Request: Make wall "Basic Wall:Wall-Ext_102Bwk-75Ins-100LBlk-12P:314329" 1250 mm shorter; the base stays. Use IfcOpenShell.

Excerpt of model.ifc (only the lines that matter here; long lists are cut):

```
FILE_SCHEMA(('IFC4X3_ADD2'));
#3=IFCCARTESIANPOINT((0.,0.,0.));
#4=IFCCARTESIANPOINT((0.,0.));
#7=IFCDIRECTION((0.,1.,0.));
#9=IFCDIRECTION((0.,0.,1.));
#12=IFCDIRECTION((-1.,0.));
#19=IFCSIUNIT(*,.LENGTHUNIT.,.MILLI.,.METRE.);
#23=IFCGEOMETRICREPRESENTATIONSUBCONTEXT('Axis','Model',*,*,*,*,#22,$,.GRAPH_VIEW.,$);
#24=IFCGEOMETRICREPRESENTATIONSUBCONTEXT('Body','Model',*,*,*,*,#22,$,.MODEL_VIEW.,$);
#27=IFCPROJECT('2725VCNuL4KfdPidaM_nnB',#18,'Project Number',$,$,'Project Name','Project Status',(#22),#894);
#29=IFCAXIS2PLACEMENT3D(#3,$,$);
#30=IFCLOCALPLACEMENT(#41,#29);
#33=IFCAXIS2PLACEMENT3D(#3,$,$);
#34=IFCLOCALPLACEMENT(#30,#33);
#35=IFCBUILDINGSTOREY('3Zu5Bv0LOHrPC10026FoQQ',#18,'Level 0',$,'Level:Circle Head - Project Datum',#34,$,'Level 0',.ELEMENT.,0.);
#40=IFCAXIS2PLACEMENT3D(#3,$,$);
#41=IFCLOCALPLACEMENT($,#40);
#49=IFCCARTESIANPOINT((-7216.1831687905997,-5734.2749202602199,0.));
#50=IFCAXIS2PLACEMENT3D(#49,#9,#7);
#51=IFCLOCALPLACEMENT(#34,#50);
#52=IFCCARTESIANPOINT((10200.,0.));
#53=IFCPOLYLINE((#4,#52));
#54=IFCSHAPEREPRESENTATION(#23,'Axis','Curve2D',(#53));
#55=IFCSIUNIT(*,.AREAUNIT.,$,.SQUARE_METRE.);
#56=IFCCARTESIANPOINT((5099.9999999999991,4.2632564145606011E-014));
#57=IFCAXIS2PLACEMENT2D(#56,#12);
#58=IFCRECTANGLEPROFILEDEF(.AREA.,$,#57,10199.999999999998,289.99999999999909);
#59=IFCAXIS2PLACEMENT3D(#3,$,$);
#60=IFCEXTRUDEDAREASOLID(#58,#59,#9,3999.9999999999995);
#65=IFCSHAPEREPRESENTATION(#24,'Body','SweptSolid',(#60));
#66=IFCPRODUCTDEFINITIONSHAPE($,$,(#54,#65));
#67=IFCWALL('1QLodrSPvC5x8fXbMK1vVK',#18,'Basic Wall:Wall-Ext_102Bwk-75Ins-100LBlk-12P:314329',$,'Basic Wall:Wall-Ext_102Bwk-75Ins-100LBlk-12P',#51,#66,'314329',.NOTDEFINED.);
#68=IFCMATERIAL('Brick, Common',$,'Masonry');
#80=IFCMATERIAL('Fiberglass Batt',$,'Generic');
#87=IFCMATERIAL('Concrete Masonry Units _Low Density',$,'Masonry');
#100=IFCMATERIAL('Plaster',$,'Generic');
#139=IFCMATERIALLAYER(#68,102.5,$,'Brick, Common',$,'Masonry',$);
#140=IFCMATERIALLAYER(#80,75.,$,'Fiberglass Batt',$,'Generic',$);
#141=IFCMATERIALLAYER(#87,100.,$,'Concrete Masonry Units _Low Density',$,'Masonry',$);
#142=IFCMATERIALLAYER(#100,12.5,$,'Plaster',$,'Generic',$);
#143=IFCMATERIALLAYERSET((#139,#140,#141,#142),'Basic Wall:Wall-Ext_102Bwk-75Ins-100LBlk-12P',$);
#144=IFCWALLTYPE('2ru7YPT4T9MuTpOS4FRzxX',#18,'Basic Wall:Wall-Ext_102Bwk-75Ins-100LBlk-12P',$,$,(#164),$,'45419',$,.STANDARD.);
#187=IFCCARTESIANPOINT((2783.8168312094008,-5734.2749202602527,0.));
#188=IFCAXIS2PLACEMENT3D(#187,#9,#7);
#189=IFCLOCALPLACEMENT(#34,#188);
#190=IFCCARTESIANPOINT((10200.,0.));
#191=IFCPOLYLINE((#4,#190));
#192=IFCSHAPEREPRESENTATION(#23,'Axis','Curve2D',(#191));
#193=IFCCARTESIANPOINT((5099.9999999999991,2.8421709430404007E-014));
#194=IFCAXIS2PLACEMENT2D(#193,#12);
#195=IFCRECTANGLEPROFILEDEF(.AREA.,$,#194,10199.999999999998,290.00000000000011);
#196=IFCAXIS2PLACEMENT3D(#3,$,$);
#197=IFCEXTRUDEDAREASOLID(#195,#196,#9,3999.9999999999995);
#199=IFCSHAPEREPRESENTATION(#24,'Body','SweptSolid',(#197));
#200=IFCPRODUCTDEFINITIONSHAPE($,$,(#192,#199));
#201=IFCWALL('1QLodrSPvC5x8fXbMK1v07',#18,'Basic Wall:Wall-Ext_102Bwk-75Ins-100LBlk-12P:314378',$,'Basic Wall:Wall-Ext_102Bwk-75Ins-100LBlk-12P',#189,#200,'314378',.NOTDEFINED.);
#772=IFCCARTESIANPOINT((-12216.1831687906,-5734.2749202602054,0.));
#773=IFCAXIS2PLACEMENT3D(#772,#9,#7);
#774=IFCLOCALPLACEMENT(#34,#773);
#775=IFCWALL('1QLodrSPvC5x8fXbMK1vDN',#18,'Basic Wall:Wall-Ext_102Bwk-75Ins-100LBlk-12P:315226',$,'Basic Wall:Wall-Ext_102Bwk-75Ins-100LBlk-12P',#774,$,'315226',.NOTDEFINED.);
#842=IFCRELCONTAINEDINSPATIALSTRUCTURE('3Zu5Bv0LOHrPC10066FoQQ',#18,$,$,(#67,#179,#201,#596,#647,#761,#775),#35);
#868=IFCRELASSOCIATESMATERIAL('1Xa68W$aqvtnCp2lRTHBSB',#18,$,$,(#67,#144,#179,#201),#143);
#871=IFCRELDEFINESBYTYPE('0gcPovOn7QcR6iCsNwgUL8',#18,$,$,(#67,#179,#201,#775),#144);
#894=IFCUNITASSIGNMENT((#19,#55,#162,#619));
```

```python
import ifcopenshell
import ifcopenshell.geom
import ifcopenshell.util.representation
import ifcopenshell.util.shape
import ifcopenshell.util.unit

model = ifcopenshell.open("model.ifc")
unit_scale = ifcopenshell.util.unit.calculate_unit_scale(model)
settings = ifcopenshell.geom.settings()


def volume(element):
    """Net volume in cubic metres, openings subtracted."""
    shape = ifcopenshell.geom.create_shape(settings, element)
    return ifcopenshell.util.shape.get_volume(shape.geometry)


wall = model.by_id(67)
before = volume(wall)

body = ifcopenshell.util.representation.get_representation(wall, "Model", "Body")
solid = body.Items[0]
old_height = solid.Depth
solid.Depth -= 1.25 / unit_scale
after = volume(wall)

print(f"height {old_height:g} -> {solid.Depth:g}, volume {before:.3f} -> {after:.3f} m3")

model.write("model-out.ifc")
```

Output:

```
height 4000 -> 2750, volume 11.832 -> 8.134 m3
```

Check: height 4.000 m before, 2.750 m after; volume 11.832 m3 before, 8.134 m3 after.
